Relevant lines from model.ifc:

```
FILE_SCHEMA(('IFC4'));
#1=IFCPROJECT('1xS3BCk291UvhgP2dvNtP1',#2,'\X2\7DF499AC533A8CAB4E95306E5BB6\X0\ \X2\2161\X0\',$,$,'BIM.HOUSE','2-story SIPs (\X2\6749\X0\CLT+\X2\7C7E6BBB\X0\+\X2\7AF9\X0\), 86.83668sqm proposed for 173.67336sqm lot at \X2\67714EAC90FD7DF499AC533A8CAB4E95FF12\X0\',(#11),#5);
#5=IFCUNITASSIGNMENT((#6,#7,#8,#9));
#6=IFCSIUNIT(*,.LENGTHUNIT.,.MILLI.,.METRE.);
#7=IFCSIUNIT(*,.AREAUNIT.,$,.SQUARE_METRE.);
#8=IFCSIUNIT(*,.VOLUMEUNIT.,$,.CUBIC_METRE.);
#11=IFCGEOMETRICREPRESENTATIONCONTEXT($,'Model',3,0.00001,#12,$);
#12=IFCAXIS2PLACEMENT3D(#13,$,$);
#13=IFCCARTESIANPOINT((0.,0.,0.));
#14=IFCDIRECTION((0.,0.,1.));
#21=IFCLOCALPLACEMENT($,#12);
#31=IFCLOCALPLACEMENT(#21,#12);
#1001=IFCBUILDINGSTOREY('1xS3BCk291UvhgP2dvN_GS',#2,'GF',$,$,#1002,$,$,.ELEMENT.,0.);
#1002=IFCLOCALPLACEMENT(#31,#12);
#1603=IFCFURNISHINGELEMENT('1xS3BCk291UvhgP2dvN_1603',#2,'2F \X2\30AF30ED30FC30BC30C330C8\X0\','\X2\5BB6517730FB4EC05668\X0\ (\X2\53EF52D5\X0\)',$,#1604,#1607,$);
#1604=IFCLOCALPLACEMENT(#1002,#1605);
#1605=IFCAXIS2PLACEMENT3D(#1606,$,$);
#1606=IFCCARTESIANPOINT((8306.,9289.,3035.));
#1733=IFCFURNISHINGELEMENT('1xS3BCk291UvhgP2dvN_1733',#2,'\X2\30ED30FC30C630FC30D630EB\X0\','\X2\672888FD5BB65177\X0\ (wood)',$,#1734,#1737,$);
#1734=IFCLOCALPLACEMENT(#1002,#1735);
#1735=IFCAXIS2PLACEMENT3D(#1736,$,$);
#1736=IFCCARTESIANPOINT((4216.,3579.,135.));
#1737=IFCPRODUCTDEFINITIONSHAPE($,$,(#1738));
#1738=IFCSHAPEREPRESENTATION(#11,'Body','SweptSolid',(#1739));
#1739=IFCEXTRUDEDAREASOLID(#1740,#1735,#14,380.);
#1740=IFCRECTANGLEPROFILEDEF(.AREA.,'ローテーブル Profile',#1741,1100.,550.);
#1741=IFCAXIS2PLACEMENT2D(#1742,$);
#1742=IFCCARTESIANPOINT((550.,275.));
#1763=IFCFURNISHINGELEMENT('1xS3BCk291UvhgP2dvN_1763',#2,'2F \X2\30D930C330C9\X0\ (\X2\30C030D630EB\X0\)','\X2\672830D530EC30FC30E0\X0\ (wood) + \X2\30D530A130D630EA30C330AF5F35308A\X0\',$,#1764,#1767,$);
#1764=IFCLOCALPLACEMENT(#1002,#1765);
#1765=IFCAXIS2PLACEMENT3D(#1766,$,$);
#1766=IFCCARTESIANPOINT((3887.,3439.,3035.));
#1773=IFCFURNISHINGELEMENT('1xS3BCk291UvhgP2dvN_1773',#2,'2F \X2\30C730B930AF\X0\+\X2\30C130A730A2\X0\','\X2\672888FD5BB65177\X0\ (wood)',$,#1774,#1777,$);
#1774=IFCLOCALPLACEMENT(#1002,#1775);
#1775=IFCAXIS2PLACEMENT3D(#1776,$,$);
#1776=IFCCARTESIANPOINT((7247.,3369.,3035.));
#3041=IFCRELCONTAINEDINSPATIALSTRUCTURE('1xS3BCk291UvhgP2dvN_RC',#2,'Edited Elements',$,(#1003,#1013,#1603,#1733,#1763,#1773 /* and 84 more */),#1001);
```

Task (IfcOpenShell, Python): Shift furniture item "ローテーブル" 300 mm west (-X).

```python
import ifcopenshell
import ifcopenshell.api.geometry
import ifcopenshell.util.placement
import ifcopenshell.util.unit

model = ifcopenshell.open("model.ifc")
unit_scale = ifcopenshell.util.unit.calculate_unit_scale(model)

item = model.by_guid("1xS3BCk291UvhgP2dvN_1733")
matrix = ifcopenshell.util.placement.get_local_placement(item.ObjectPlacement)
matrix[0, 3] -= 0.3 / unit_scale
ifcopenshell.api.geometry.edit_object_placement(model, product=item, matrix=matrix, is_si=False)

print(ifcopenshell.util.placement.get_local_placement(item.ObjectPlacement).round(3) + 0.0)

model.write("model_updated.ifc")
```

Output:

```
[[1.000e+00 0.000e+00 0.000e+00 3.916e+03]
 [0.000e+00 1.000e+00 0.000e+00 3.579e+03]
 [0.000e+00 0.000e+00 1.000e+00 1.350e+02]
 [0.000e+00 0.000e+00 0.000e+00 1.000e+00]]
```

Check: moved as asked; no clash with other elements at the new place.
